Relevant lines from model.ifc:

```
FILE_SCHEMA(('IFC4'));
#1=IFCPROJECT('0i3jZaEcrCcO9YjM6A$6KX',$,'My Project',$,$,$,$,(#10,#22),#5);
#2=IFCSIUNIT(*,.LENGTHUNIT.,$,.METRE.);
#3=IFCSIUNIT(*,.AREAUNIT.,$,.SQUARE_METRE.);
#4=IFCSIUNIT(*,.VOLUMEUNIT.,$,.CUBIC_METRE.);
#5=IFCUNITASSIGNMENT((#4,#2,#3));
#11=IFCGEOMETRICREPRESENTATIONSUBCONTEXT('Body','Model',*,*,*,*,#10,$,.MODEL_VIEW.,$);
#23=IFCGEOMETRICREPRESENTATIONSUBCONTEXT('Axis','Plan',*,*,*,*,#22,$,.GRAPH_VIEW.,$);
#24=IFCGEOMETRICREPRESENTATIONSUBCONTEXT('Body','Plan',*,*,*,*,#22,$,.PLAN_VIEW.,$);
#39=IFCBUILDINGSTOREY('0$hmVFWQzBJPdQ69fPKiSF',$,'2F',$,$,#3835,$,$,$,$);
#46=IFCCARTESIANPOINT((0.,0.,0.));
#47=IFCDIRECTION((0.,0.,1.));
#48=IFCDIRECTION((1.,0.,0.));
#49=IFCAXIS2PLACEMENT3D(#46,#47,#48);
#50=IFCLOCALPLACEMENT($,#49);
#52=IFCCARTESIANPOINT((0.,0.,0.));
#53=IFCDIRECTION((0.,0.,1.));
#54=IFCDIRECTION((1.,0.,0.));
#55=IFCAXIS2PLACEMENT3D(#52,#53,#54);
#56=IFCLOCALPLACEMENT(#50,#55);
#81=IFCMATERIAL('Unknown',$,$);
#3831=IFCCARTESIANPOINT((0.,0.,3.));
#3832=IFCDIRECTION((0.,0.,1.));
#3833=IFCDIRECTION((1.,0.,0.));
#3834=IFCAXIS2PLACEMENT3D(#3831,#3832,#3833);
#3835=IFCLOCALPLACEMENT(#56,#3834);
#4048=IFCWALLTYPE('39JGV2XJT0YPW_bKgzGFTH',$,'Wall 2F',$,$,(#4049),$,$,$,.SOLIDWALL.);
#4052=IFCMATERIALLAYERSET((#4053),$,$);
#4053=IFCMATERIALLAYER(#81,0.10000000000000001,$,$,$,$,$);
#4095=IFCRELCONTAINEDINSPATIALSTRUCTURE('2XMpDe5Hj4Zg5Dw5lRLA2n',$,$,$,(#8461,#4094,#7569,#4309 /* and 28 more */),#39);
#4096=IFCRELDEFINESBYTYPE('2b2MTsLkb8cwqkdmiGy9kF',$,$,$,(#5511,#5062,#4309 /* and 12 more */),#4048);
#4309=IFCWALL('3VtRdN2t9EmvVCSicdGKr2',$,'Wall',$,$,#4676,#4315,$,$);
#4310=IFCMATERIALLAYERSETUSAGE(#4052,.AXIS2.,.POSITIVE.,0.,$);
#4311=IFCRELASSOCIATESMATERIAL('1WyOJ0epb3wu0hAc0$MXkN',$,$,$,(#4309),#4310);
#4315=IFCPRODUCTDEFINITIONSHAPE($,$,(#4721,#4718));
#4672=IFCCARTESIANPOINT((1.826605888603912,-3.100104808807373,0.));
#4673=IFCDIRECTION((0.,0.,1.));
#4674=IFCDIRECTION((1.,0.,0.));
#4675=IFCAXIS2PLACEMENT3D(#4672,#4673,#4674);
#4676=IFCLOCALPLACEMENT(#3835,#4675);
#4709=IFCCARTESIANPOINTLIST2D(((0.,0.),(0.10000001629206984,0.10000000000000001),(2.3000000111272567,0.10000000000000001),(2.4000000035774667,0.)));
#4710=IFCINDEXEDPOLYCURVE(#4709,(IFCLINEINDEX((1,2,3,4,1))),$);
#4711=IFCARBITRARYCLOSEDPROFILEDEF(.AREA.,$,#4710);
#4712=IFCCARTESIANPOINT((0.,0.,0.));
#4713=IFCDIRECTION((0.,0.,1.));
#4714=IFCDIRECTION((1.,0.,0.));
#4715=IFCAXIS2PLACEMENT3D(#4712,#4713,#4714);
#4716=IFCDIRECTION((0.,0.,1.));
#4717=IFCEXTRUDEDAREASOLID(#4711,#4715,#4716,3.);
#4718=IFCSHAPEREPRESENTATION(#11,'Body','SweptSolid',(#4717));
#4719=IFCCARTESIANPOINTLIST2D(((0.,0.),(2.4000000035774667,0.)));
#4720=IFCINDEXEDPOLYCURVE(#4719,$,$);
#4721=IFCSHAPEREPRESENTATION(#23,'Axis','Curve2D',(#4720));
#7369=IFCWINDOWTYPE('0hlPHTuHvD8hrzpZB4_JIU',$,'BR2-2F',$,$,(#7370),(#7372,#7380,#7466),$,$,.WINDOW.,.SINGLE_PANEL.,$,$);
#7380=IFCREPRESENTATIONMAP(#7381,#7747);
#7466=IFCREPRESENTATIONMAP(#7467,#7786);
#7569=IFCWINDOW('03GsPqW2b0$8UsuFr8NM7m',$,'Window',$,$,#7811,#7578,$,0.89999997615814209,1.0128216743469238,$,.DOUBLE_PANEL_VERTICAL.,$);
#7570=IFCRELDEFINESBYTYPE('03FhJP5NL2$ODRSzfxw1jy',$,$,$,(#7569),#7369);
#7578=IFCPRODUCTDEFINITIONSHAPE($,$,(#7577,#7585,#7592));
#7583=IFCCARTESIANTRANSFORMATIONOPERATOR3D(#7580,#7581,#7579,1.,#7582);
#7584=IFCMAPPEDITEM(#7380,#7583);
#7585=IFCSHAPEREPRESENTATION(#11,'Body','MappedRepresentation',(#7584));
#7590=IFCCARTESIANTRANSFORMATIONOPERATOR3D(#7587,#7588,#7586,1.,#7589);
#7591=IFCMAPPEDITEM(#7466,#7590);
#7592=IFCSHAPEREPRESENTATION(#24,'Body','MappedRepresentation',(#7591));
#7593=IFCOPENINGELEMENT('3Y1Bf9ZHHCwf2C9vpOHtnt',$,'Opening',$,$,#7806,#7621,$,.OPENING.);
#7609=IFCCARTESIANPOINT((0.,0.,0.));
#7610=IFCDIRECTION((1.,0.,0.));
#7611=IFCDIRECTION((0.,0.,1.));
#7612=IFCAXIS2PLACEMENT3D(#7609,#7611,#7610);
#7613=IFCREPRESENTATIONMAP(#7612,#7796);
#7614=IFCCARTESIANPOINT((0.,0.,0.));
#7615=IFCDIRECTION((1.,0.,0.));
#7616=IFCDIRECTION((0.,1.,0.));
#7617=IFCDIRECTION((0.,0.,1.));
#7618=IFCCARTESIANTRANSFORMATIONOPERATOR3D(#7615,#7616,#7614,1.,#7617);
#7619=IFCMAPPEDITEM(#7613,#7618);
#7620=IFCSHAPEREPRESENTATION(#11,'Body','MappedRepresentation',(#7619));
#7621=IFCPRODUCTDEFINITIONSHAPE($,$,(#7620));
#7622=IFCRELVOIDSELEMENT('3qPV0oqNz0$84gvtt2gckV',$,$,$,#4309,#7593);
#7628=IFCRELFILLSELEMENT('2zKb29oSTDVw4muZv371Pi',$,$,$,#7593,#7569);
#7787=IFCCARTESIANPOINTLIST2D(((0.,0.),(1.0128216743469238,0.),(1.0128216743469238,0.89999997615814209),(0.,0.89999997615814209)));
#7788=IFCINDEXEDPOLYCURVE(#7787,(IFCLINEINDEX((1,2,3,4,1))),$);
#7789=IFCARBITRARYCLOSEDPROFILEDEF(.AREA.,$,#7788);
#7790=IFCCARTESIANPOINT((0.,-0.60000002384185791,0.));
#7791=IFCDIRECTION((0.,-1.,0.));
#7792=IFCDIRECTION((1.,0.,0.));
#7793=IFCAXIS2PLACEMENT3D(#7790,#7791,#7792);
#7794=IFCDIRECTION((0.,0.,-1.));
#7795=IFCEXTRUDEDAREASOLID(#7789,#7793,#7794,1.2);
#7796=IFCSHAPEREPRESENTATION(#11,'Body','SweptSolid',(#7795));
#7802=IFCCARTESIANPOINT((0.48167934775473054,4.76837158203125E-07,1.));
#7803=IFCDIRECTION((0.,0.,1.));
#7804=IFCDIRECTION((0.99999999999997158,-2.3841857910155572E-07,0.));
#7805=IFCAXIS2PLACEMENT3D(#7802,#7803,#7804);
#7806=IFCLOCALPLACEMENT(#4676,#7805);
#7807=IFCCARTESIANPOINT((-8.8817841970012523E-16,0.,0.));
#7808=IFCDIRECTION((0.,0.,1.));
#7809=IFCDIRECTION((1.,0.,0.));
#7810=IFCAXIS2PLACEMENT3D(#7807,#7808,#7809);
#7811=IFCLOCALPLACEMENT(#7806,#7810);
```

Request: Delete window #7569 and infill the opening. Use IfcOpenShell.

```python
import ifcopenshell
import ifcopenshell.api.feature
import ifcopenshell.api.root
import ifcopenshell.geom
import ifcopenshell.util.shape

model = ifcopenshell.open("model.ifc")
settings = ifcopenshell.geom.settings()


def volume(element):
    """Net volume in cubic metres, openings subtracted."""
    shape = ifcopenshell.geom.create_shape(settings, element)
    return ifcopenshell.util.shape.get_volume(shape.geometry)


window = model.by_guid("03GsPqW2b0$8UsuFr8NM7m")
opening = window.FillsVoids[0].RelatingOpeningElement
wall = opening.VoidsElements[0].RelatingBuildingElement
before = volume(wall)

ifcopenshell.api.root.remove_product(model, product=window)
ifcopenshell.api.feature.remove_feature(model, feature=opening)

after = volume(wall)

print(f"wall volume {before:.3f} -> {after:.3f} m3")

model.write("model_updated.ifc")
```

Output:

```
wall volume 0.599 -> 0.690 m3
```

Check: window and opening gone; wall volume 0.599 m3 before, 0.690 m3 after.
